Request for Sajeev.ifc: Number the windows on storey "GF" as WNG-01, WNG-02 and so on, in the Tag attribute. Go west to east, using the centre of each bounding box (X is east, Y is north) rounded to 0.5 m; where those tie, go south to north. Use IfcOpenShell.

First a look at what the model holds.

```python
import ifcopenshell
import ifcopenshell.util.element
import ifcopenshell.util.placement

model = ifcopenshell.open("Sajeev.ifc")
print(model.schema)
storey = next(s for s in model.by_type("IfcBuildingStorey") if s.Name == "GF")
windows = [e for e in ifcopenshell.util.element.get_decomposition(storey) if e.is_a("IfcWindow")]
for e in sorted(windows, key=lambda e: e.id()):
    origin = ifcopenshell.util.placement.get_local_placement(e.ObjectPlacement)[:3, 3]
    print(e.id(), e.Tag, e.Name, origin.round(2) + 0.0, sep=" | ")
```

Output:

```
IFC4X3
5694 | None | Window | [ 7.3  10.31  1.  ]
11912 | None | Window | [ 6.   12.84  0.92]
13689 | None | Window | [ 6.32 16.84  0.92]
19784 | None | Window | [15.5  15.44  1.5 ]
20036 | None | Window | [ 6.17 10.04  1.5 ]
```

```python
import ifcopenshell
import ifcopenshell.geom
import ifcopenshell.util.element
import ifcopenshell.util.shape

model = ifcopenshell.open("Sajeev.ifc")
settings = ifcopenshell.geom.settings()
settings.set("use-world-coords", True)


def centre(element):
    shape = ifcopenshell.geom.create_shape(settings, element)
    return ifcopenshell.util.shape.get_bbox_centroid(shape.geometry)


storey = next(s for s in model.by_type("IfcBuildingStorey") if s.Name == "GF")
windows = [e for e in ifcopenshell.util.element.get_decomposition(storey) if e.is_a("IfcWindow")]

# Insertion points can sit at a corner or the storey origin, so sort by the geometry (in metres).
centres = {e: centre(e) for e in windows}
windows.sort(key=lambda e: (round(centres[e][0] / 0.5), centres[e][1]))

for i, e in enumerate(windows, start=1):
    number = f"WNG-{i:02d}"
    e.Tag = number
    print(e.id(), number)

model.write("Sajeev_v2.ifc")
```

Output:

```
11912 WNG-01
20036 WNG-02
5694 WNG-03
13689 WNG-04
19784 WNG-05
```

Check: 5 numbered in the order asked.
